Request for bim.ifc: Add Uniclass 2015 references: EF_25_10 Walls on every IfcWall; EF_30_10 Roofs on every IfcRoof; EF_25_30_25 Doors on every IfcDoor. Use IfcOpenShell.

First a look at what the model holds.

```python
import ifcopenshell

model = ifcopenshell.open("bim.ifc")
print(model.schema)
print("classifications:", [c.Name for c in model.by_type("IfcClassification")])
for ifc_class in ("IfcDoor", "IfcRoof", "IfcStair", "IfcWall", "IfcWindow"):
    print(ifc_class, len(model.by_type(ifc_class)))
```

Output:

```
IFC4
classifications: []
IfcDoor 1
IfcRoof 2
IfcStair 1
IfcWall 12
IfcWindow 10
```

```python
import ifcopenshell
import ifcopenshell.api.classification

model = ifcopenshell.open("bim.ifc")

system = ifcopenshell.api.classification.add_classification(model, classification="Uniclass 2015")

codes = {
    "IfcWall": ("EF_25_10", "Walls"),
    "IfcRoof": ("EF_30_10", "Roofs"),
    "IfcDoor": ("EF_25_30_25", "Doors"),
}
for ifc_class, (code, name) in codes.items():
    products = model.by_type(ifc_class)
    ifcopenshell.api.classification.add_reference(
        model, products=products, classification=system, identification=code, name=name
    )
    print(code, len(products))

model.write("bim_updated.ifc")
```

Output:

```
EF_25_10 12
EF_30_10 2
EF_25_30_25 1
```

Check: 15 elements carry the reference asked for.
